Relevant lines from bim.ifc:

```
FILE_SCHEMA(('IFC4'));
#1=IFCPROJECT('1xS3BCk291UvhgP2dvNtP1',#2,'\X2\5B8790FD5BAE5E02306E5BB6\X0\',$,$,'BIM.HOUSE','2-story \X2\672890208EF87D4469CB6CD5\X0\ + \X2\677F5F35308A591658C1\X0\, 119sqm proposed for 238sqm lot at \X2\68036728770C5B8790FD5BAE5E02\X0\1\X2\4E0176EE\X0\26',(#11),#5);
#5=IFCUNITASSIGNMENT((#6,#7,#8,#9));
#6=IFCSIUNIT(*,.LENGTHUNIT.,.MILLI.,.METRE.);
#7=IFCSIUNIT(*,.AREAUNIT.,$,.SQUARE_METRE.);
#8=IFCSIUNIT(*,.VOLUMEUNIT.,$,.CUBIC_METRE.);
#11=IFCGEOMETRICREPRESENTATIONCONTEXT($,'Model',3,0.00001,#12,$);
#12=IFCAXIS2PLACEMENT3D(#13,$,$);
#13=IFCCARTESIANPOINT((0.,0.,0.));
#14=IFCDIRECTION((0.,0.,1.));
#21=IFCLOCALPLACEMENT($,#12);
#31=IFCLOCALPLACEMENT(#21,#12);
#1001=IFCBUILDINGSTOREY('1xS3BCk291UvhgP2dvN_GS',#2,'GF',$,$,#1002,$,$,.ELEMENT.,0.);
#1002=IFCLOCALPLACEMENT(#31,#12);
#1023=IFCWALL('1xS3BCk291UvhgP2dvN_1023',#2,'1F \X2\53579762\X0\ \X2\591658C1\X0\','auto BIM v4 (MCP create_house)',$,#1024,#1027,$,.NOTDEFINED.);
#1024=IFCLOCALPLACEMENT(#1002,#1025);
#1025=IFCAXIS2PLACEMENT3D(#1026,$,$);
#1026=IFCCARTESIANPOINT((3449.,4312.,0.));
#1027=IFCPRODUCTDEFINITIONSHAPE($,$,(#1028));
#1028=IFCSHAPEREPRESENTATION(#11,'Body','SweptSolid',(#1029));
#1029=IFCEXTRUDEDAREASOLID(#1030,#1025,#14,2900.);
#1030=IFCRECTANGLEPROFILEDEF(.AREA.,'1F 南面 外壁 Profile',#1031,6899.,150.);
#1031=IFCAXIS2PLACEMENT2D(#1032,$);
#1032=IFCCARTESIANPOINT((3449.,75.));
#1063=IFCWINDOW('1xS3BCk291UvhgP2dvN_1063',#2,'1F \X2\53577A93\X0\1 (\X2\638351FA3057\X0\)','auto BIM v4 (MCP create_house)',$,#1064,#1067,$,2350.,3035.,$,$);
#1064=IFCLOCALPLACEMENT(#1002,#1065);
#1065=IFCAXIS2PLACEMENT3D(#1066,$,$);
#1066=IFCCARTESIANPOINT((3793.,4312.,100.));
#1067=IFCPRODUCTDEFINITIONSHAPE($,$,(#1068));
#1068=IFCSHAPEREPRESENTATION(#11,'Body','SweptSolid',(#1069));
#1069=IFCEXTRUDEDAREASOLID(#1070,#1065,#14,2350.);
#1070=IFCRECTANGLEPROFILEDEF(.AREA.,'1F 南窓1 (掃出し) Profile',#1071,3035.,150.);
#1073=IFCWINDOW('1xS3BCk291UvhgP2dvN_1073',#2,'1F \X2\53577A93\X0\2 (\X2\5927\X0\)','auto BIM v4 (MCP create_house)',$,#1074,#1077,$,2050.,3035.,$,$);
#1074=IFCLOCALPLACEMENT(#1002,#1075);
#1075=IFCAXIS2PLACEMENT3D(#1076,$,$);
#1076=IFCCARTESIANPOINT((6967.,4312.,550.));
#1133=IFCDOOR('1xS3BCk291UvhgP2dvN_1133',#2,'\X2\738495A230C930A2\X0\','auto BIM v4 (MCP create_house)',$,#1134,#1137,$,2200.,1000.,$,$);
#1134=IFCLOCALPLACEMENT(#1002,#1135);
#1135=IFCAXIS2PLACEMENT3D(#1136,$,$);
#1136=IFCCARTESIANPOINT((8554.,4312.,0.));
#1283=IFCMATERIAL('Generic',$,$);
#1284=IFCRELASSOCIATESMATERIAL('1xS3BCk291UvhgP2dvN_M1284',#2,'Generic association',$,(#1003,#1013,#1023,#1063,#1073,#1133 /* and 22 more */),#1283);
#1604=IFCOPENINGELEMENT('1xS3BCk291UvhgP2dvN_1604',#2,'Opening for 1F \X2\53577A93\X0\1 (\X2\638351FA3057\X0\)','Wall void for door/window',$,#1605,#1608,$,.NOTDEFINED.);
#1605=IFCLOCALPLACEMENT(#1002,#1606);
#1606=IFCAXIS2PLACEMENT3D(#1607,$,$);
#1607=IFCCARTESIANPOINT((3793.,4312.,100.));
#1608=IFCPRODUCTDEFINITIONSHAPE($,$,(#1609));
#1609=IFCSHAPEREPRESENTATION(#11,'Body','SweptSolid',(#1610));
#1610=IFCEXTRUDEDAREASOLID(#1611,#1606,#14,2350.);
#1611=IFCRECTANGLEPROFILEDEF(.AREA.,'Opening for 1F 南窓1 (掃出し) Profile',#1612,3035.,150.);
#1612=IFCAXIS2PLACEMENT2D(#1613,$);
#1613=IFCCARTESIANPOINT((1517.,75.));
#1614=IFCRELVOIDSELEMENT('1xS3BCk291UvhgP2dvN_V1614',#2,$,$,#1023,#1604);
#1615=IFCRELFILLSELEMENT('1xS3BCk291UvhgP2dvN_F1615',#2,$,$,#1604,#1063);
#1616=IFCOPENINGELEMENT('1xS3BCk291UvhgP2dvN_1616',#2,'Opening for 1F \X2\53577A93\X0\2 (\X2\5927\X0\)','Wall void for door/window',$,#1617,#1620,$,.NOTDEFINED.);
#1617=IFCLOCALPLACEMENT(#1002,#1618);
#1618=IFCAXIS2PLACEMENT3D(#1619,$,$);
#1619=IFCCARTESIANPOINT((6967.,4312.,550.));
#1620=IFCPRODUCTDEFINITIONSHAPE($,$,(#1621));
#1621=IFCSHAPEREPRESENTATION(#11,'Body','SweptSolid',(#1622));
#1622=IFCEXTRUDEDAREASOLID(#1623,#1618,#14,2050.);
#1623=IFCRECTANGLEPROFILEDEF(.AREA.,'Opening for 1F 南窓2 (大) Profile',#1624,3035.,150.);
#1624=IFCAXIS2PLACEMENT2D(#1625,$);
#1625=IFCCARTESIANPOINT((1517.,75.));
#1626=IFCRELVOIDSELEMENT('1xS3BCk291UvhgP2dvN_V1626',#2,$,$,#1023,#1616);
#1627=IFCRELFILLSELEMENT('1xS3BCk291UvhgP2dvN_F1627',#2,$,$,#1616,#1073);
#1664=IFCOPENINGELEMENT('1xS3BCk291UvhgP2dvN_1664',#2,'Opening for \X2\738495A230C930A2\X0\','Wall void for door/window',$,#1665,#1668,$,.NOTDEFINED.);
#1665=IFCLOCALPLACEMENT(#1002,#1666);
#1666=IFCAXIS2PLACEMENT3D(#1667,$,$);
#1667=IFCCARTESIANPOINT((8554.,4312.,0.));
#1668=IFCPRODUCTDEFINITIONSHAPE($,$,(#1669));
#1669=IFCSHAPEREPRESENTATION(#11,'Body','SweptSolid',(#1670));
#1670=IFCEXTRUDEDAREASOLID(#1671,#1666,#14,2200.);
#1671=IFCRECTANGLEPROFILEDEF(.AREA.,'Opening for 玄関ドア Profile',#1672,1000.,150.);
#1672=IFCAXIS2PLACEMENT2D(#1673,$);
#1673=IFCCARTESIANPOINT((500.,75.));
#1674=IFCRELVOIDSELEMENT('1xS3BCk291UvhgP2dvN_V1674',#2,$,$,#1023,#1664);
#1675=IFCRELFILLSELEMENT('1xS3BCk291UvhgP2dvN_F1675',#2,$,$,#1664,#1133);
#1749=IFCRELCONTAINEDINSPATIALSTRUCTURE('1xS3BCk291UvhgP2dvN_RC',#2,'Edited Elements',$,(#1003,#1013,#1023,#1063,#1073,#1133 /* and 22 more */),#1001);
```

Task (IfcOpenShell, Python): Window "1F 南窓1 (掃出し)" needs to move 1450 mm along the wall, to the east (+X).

```python
import ifcopenshell
import ifcopenshell.api.geometry
import ifcopenshell.util.placement
import ifcopenshell.util.unit

model = ifcopenshell.open("bim.ifc")
unit_scale = ifcopenshell.util.unit.calculate_unit_scale(model)

window = model.by_guid("1xS3BCk291UvhgP2dvN_1063")
opening = window.FillsVoids[0].RelatingOpeningElement
wall = opening.VoidsElements[0].RelatingBuildingElement

wall_matrix = ifcopenshell.util.placement.get_local_placement(wall.ObjectPlacement)
shift = wall_matrix[:3, 0] * 1.45 / unit_scale
before = ifcopenshell.util.placement.get_local_placement(window.ObjectPlacement)[:3, 3].copy()

# The window is not placed relative to its opening, so move both.
for product in (opening, window):
    matrix = ifcopenshell.util.placement.get_local_placement(product.ObjectPlacement)
    matrix[:3, 3] += shift
    ifcopenshell.api.geometry.edit_object_placement(model, product=product, matrix=matrix, is_si=False)

after = ifcopenshell.util.placement.get_local_placement(window.ObjectPlacement)[:3, 3]
print("window moved by", (after - before).round(3) + 0.0)

model.write("bim_edited.ifc")
```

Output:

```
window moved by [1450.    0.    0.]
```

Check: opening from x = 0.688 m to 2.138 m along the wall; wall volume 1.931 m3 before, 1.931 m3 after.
